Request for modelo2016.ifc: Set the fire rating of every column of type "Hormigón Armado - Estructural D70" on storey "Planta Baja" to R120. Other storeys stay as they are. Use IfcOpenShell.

First a look at what the model holds.

```python
import ifcopenshell
import ifcopenshell.util.element

model = ifcopenshell.open("modelo2016.ifc")
print(model.schema)
storey = next(s for s in model.by_type("IfcBuildingStorey") if s.Name == "Planta Baja")
columns = [e for e in ifcopenshell.util.element.get_decomposition(storey) if e.is_a("IfcColumn")]
seen = {}
for e in columns:
    element_type = ifcopenshell.util.element.get_type(e)
    key = (element_type.Name if element_type != e and element_type else None, ifcopenshell.util.element.get_pset(e, "Pset_ColumnCommon", "FireRating"))
    seen[key] = seen.get(key, 0) + 1
for (name, value), count in sorted(seen.items(), key=str):
    print(count, "x", name, "|", value)
```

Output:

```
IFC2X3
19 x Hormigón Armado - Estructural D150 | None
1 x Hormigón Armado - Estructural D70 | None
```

```python
import ifcopenshell
import ifcopenshell.api.pset
import ifcopenshell.util.element

model = ifcopenshell.open("modelo2016.ifc")

storey = next(s for s in model.by_type("IfcBuildingStorey") if s.Name == "Planta Baja")
columns = [e for e in ifcopenshell.util.element.get_decomposition(storey) if e.is_a("IfcColumn")]

count = 0
for e in columns:
    element_type = ifcopenshell.util.element.get_type(e)
    if element_type in (None, e) or element_type.Name != "Hormigón Armado - Estructural D70":
        continue
    # add_pset returns the element's existing set when there is one.
    pset = ifcopenshell.api.pset.add_pset(model, product=e, name="Pset_ColumnCommon")
    ifcopenshell.api.pset.edit_pset(model, pset=pset, properties={"FireRating": "R120"})
    count += 1

print(count, "columns updated")

model.write("modelo2016_updated.ifc")
```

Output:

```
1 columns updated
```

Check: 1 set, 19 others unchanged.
